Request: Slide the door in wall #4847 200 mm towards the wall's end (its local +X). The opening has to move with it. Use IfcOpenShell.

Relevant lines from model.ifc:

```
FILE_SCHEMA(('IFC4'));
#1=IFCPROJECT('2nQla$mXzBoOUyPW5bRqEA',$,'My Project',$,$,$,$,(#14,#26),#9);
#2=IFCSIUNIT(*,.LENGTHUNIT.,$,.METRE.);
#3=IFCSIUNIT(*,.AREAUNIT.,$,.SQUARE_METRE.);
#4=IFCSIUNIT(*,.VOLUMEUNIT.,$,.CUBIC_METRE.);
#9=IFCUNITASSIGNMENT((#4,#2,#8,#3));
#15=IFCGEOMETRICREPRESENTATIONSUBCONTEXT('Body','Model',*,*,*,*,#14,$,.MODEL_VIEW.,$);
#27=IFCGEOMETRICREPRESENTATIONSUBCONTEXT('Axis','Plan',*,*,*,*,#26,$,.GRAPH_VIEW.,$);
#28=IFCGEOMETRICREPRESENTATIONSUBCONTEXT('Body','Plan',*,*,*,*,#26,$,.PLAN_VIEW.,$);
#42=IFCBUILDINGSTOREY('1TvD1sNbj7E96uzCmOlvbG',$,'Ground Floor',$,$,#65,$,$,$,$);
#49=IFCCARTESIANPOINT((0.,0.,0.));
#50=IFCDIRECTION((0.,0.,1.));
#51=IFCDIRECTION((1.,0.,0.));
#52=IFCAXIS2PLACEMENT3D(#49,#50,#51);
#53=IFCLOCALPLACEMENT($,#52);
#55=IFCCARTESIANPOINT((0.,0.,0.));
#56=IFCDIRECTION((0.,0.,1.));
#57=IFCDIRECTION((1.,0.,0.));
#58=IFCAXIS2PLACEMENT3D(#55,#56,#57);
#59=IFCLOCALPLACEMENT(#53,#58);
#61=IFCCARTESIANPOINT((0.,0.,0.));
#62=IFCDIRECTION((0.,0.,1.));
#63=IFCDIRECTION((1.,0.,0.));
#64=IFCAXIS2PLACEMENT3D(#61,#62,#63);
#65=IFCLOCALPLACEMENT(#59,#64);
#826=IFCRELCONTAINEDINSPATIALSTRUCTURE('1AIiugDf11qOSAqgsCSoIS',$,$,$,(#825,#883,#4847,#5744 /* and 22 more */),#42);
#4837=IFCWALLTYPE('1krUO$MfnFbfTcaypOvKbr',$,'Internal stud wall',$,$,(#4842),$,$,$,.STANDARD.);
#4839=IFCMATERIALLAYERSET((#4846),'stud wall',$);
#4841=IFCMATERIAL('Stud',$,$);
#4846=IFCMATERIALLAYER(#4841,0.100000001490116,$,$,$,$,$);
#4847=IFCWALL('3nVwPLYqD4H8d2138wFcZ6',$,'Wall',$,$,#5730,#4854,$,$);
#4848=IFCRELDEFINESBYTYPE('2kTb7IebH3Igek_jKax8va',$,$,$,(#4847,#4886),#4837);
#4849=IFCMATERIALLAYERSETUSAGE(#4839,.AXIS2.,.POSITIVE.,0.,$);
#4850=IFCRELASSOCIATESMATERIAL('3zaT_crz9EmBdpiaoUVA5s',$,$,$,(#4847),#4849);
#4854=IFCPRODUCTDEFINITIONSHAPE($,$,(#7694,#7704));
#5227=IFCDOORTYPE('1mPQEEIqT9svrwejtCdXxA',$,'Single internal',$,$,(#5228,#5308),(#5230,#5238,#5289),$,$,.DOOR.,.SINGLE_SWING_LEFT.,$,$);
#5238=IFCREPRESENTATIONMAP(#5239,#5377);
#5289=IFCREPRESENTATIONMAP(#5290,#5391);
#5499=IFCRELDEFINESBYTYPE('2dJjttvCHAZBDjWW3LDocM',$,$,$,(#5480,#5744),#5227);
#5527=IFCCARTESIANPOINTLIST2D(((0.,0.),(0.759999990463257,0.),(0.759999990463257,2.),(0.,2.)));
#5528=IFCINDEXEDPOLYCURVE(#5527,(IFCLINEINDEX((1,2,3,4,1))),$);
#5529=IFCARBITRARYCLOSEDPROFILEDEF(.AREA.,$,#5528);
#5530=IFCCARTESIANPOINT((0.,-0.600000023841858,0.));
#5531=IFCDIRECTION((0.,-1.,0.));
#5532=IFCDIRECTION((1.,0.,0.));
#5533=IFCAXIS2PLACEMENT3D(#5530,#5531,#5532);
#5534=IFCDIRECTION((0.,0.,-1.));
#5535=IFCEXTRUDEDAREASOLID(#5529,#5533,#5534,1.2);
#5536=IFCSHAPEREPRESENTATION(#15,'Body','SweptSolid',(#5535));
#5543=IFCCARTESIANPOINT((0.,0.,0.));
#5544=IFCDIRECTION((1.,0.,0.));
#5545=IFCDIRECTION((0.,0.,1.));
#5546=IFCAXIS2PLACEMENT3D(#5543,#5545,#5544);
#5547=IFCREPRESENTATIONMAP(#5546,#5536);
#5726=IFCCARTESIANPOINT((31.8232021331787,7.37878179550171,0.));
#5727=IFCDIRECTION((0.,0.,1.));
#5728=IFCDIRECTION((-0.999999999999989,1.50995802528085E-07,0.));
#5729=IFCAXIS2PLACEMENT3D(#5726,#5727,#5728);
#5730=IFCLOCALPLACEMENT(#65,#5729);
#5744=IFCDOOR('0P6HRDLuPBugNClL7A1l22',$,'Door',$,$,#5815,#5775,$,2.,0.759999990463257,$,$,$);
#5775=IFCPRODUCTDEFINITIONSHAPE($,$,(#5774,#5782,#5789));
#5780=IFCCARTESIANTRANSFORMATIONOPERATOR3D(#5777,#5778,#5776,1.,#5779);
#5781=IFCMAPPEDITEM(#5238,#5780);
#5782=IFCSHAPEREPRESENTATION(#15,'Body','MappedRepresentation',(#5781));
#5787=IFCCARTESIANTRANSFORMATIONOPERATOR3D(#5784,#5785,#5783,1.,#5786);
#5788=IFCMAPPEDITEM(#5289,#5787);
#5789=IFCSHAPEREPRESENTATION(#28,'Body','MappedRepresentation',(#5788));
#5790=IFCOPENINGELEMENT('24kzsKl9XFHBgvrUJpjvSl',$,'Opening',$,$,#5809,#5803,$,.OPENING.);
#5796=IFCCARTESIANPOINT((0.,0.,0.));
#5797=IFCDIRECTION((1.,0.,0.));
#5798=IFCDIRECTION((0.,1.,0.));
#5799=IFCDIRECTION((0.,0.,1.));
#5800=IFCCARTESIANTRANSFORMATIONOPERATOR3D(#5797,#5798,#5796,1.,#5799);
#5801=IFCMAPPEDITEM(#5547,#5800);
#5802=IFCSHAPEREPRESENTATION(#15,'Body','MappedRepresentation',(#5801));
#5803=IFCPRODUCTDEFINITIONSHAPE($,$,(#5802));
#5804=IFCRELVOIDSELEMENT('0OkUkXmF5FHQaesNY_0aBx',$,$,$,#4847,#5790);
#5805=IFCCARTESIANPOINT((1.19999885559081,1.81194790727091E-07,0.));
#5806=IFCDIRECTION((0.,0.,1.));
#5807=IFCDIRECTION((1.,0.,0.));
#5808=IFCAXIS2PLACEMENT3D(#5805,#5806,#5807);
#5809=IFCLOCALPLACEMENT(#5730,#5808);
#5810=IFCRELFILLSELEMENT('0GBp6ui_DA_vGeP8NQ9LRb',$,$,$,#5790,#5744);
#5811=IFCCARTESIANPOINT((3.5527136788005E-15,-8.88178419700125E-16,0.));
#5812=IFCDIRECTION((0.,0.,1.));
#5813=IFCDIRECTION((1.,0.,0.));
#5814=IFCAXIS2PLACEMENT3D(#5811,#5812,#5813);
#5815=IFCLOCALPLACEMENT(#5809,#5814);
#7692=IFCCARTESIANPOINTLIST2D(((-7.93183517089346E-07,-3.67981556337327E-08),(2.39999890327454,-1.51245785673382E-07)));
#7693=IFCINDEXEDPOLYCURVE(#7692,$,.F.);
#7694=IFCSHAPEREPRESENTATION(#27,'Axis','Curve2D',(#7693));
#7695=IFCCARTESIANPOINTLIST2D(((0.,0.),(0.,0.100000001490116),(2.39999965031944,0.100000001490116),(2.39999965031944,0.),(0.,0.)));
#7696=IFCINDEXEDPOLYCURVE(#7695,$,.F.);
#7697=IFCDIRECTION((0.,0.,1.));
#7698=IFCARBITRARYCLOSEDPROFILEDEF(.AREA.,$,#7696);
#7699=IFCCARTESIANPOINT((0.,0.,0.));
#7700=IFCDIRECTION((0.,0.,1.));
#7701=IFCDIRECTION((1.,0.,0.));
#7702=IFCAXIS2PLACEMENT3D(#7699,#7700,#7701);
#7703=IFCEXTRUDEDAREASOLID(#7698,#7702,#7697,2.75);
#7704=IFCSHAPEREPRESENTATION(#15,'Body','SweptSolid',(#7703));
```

```python
import ifcopenshell
import ifcopenshell.api.geometry
import ifcopenshell.util.placement

model = ifcopenshell.open("model.ifc")

door = model.by_id(5744)
opening = door.FillsVoids[0].RelatingOpeningElement
wall = opening.VoidsElements[0].RelatingBuildingElement

wall_matrix = ifcopenshell.util.placement.get_local_placement(wall.ObjectPlacement)
shift = wall_matrix[:3, 0] * 0.2
before = ifcopenshell.util.placement.get_local_placement(door.ObjectPlacement)[:3, 3].copy()

# The door is placed relative to its opening, so it follows when the opening moves.
matrix = ifcopenshell.util.placement.get_local_placement(opening.ObjectPlacement)
matrix[:3, 3] += shift
ifcopenshell.api.geometry.edit_object_placement(
    model, product=opening, matrix=matrix, is_si=False, should_transform_children=True
)

after = ifcopenshell.util.placement.get_local_placement(door.ObjectPlacement)[:3, 3]
print("door moved by", (after - before).round(3) + 0.0)

model.write("model_updated.ifc")
```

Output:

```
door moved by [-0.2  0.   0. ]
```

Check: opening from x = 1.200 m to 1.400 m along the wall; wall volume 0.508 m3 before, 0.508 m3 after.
